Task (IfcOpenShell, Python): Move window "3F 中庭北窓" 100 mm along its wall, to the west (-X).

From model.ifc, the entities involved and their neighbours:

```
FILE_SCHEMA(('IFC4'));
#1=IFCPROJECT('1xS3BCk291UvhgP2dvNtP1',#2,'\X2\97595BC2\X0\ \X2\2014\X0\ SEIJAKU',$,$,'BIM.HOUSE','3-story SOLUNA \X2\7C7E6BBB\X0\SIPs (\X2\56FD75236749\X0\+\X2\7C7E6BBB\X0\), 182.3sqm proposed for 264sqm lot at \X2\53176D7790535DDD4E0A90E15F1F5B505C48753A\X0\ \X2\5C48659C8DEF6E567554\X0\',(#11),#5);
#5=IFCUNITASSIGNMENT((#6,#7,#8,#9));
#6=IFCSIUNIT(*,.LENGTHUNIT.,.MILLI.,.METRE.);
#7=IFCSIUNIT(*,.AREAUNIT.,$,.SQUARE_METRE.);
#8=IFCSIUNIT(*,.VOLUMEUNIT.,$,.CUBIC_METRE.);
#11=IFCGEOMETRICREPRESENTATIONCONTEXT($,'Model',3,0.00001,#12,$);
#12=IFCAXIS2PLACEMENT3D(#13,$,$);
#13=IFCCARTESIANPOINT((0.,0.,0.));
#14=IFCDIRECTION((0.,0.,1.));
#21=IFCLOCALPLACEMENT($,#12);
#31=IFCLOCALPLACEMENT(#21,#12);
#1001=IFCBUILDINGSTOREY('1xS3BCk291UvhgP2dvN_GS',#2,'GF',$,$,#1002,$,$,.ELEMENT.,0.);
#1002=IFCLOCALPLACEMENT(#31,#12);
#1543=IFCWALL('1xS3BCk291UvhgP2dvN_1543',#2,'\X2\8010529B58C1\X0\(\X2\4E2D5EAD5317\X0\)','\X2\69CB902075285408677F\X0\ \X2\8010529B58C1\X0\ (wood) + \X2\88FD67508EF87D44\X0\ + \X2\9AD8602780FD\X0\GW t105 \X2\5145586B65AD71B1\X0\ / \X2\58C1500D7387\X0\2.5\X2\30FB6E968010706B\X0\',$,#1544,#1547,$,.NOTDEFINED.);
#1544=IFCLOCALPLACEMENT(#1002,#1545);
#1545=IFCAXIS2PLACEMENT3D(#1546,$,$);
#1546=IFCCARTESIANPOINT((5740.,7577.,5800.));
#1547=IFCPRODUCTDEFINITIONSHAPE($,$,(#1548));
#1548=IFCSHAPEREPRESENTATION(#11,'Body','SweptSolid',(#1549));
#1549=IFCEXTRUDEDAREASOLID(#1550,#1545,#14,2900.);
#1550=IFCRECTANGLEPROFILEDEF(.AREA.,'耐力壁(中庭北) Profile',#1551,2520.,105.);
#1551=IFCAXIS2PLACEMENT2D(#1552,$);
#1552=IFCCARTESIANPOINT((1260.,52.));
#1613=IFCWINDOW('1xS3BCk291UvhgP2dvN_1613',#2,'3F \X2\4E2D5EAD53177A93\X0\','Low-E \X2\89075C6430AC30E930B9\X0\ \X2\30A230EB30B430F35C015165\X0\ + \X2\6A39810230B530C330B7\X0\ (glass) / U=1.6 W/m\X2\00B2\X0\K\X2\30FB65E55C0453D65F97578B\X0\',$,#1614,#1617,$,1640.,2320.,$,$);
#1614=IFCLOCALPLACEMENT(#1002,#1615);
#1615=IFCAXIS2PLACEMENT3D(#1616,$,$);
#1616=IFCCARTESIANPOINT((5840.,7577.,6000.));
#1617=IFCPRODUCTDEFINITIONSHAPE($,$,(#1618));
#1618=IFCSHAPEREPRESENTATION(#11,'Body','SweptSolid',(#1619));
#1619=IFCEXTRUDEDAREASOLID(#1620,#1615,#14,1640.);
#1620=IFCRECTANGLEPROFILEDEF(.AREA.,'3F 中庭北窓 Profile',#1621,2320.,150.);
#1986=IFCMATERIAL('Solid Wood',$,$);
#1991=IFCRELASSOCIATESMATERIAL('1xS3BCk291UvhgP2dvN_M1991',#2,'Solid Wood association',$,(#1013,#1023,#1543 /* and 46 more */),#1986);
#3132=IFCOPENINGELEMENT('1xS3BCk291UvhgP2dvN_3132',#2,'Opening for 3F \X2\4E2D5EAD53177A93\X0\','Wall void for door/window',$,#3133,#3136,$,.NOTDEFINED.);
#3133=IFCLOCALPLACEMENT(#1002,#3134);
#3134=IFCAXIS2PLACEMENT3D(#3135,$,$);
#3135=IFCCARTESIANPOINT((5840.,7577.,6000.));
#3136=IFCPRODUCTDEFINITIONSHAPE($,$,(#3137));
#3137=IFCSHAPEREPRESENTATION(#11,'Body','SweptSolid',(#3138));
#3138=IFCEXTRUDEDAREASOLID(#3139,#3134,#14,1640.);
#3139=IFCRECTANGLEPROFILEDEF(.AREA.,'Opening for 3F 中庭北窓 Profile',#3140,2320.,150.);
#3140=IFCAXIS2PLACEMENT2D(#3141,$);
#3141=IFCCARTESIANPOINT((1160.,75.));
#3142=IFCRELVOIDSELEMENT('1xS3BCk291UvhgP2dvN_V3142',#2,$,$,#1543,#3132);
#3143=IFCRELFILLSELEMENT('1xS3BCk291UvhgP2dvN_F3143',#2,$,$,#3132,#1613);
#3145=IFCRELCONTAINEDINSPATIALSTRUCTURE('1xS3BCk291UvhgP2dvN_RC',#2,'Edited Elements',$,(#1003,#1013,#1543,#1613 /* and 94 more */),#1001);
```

```python
import ifcopenshell
import ifcopenshell.api.geometry
import ifcopenshell.util.placement

model = ifcopenshell.open("model.ifc")

window = model.by_guid("1xS3BCk291UvhgP2dvN_1613")
opening = window.FillsVoids[0].RelatingOpeningElement
wall = opening.VoidsElements[0].RelatingBuildingElement

wall_matrix = ifcopenshell.util.placement.get_local_placement(wall.ObjectPlacement)
shift = wall_matrix[:3, 0] * -100.0
before = ifcopenshell.util.placement.get_local_placement(window.ObjectPlacement)[:3, 3].copy()

# The window is not placed relative to its opening, so move both.
for product in (opening, window):
    matrix = ifcopenshell.util.placement.get_local_placement(product.ObjectPlacement)
    matrix[:3, 3] += shift
    ifcopenshell.api.geometry.edit_object_placement(model, product=product, matrix=matrix, is_si=False)

after = ifcopenshell.util.placement.get_local_placement(window.ObjectPlacement)[:3, 3]
print("window moved by", (after - before).round(3) + 0.0)

model.write("model_rev.ifc")
```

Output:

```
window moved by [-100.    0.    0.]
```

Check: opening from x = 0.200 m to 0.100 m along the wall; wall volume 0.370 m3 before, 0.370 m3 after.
